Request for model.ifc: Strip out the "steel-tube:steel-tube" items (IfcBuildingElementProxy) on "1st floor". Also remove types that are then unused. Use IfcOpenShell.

First a look at what the model holds.

```python
import ifcopenshell
import ifcopenshell.util.element

model = ifcopenshell.open("model.ifc")
print(model.schema)
storey = next(s for s in model.by_type("IfcBuildingStorey") if s.Name == "1st floor")
proxies = [e for e in ifcopenshell.util.element.get_decomposition(storey) if e.is_a("IfcBuildingElementProxy")]
seen = {}
for e in proxies:
    element_type = ifcopenshell.util.element.get_type(e)
    name = element_type.Name if element_type not in (None, e) else None
    seen[name] = seen.get(name, 0) + 1
for name, count in sorted(seen.items(), key=str):
    print(count, "x", name)
```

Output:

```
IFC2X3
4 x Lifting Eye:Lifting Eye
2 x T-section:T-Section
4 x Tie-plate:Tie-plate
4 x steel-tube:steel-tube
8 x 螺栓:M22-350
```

```python
import ifcopenshell
import ifcopenshell.api.root
import ifcopenshell.util.element

model = ifcopenshell.open("model.ifc")

storey = next(s for s in model.by_type("IfcBuildingStorey") if s.Name == "1st floor")
proxies = [e for e in ifcopenshell.util.element.get_decomposition(storey) if e.is_a("IfcBuildingElementProxy")]
targets = [e for e in proxies if (t := ifcopenshell.util.element.get_type(e)) not in (None, e) and t.Name == "steel-tube:steel-tube"]
types = {ifcopenshell.util.element.get_type(e) for e in targets} - {None, *targets}

for e in targets:
    ifcopenshell.api.root.remove_product(model, product=e)
print(len(targets), "removed")

unused = [t for t in types if not ifcopenshell.util.element.get_types(t)]
for t in unused:
    ifcopenshell.api.root.remove_product(model, product=t)
print(len(unused), "unused types removed")

model.write("model_v2.ifc")
```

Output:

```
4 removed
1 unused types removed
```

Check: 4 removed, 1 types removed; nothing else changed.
